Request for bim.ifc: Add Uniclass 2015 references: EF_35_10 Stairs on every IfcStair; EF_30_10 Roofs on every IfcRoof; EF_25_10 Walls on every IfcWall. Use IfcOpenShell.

First a look at what the model holds.

```python
import ifcopenshell

model = ifcopenshell.open("bim.ifc")
print(model.schema)
print("classifications:", [c.Name for c in model.by_type("IfcClassification")])
for ifc_class in ("IfcDoor", "IfcRoof", "IfcStair", "IfcWall", "IfcWindow"):
    print(ifc_class, len(model.by_type(ifc_class)))
```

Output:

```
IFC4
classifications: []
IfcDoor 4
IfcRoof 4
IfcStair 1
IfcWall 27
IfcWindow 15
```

```python
import ifcopenshell
import ifcopenshell.api.classification

model = ifcopenshell.open("bim.ifc")

system = ifcopenshell.api.classification.add_classification(model, classification="Uniclass 2015")

codes = {
    "IfcStair": ("EF_35_10", "Stairs"),
    "IfcRoof": ("EF_30_10", "Roofs"),
    "IfcWall": ("EF_25_10", "Walls"),
}
for ifc_class, (code, name) in codes.items():
    products = model.by_type(ifc_class)
    ifcopenshell.api.classification.add_reference(
        model, products=products, classification=system, identification=code, name=name
    )
    print(code, len(products))

model.write("bim_v2.ifc")
```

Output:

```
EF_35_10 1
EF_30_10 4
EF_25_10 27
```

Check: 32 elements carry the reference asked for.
